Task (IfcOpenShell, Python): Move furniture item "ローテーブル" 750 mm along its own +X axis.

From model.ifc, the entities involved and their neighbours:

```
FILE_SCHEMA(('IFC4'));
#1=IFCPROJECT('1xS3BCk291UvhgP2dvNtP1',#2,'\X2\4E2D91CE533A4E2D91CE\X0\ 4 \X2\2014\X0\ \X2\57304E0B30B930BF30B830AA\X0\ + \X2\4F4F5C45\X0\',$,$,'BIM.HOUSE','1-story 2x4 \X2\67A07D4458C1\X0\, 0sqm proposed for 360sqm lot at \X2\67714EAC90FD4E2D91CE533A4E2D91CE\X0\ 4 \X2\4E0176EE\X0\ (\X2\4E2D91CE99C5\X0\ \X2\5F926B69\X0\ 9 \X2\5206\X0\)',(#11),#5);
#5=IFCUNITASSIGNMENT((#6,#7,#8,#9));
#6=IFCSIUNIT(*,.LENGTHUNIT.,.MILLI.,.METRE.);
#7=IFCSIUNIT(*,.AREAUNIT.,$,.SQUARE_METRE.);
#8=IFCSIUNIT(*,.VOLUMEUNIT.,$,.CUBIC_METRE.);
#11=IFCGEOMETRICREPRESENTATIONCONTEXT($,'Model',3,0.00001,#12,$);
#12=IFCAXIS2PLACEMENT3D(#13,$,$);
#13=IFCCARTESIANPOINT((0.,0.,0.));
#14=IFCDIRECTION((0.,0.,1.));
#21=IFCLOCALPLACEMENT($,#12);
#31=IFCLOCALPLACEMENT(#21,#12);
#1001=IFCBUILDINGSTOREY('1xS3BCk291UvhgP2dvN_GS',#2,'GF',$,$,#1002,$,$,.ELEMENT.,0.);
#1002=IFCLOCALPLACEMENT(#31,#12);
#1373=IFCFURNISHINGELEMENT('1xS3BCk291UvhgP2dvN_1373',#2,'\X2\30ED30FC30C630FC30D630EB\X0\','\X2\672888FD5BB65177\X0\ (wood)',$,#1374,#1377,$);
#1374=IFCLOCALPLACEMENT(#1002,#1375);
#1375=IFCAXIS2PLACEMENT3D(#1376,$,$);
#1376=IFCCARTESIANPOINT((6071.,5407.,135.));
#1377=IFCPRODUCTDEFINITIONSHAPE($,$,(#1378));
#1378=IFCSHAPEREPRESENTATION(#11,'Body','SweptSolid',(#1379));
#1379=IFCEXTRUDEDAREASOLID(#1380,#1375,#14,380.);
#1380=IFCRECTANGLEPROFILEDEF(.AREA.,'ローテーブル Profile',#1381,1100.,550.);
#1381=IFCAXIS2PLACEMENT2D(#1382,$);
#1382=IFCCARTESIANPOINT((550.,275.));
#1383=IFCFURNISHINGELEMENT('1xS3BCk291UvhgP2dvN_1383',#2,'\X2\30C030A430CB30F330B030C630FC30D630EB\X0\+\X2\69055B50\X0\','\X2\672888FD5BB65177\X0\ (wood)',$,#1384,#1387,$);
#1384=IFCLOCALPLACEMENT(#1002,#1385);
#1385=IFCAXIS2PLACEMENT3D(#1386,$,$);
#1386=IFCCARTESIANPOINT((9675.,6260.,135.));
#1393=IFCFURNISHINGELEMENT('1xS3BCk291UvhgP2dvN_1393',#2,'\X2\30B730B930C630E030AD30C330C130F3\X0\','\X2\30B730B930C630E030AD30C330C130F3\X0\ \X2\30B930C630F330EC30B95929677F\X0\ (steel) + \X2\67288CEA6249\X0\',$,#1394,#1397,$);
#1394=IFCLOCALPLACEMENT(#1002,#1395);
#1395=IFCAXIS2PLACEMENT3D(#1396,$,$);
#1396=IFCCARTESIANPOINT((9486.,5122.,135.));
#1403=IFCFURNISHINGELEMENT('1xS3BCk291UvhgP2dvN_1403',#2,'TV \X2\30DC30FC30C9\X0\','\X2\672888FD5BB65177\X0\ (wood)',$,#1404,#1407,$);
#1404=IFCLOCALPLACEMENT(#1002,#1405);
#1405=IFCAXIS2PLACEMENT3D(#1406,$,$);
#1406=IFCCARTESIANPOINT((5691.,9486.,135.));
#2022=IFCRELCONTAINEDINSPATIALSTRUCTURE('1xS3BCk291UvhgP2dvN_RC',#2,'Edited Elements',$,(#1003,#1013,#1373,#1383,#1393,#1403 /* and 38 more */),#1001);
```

```python
import ifcopenshell
import ifcopenshell.api.geometry
import ifcopenshell.util.placement

model = ifcopenshell.open("model.ifc")

item = model.by_id(1373)
matrix = ifcopenshell.util.placement.get_local_placement(item.ObjectPlacement)
matrix[:3, 3] += matrix[:3, 0] * 750.0
ifcopenshell.api.geometry.edit_object_placement(model, product=item, matrix=matrix, is_si=False)

print(ifcopenshell.util.placement.get_local_placement(item.ObjectPlacement).round(3) + 0.0)

model.write("model_v2.ifc")
```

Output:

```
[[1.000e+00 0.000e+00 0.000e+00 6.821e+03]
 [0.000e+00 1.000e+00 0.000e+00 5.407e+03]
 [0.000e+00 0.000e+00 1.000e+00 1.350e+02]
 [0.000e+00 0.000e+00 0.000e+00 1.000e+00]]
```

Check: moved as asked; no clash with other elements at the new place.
